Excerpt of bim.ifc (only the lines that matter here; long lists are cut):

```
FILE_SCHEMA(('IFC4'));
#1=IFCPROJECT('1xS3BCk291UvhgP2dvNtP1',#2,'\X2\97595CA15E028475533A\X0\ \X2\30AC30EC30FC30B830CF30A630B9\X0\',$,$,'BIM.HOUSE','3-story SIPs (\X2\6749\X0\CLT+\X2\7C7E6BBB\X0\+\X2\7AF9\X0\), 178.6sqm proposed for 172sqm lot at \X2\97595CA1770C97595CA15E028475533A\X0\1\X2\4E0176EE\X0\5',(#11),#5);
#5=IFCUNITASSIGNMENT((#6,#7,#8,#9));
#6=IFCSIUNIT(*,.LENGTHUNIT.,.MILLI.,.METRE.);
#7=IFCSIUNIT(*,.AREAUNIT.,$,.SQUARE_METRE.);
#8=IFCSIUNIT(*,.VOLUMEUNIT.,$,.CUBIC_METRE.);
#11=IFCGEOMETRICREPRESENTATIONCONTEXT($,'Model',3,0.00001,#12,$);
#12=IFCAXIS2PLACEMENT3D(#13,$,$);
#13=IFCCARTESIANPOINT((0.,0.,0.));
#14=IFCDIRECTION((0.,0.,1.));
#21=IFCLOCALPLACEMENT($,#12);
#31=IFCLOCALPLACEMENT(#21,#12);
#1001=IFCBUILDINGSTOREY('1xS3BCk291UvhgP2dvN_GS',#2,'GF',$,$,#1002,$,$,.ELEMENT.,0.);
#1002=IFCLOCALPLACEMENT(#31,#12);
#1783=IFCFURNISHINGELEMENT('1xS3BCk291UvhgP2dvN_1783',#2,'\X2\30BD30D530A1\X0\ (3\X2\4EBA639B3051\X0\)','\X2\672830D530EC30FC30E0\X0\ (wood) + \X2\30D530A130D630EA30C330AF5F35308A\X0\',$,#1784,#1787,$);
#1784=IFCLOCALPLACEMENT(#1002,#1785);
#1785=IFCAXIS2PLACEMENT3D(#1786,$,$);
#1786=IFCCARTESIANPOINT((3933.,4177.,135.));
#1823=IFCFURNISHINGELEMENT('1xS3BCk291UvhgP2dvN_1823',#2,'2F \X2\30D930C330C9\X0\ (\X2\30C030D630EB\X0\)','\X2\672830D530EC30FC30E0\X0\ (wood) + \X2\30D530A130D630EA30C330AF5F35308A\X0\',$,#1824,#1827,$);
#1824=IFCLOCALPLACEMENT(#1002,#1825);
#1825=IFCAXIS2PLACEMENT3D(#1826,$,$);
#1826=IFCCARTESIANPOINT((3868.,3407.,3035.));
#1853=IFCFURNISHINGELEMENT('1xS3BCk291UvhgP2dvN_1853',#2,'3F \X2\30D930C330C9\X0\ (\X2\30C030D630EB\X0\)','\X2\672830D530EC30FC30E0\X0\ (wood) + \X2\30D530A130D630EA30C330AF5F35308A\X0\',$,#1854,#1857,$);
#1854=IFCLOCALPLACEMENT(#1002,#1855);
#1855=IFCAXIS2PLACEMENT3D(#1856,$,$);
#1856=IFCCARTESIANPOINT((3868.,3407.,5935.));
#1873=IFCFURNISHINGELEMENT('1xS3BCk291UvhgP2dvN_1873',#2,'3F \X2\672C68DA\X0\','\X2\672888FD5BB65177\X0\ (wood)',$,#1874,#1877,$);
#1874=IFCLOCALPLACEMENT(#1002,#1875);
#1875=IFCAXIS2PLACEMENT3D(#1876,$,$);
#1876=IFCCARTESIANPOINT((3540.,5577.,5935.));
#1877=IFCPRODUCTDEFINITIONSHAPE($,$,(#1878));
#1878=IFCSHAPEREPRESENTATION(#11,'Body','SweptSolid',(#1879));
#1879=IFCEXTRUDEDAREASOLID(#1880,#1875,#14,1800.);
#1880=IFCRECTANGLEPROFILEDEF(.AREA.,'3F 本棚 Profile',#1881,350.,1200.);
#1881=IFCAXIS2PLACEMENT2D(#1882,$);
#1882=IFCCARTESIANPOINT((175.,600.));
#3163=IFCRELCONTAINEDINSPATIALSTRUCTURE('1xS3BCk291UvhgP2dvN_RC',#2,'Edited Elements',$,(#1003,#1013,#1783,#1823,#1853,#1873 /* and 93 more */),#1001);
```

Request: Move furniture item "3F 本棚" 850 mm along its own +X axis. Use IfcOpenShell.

```python
import ifcopenshell
import ifcopenshell.api.geometry
import ifcopenshell.util.placement
import ifcopenshell.util.unit

model = ifcopenshell.open("bim.ifc")
unit_scale = ifcopenshell.util.unit.calculate_unit_scale(model)

item = model.by_guid("1xS3BCk291UvhgP2dvN_1873")
matrix = ifcopenshell.util.placement.get_local_placement(item.ObjectPlacement)
matrix[:3, 3] += matrix[:3, 0] * 0.85 / unit_scale
ifcopenshell.api.geometry.edit_object_placement(model, product=item, matrix=matrix, is_si=False)

print(ifcopenshell.util.placement.get_local_placement(item.ObjectPlacement).round(3) + 0.0)

model.write("bim-out.ifc")
```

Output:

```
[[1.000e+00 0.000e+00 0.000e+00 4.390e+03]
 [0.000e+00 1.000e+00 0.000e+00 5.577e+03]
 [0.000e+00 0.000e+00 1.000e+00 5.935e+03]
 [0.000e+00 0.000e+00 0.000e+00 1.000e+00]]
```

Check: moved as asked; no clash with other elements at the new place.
